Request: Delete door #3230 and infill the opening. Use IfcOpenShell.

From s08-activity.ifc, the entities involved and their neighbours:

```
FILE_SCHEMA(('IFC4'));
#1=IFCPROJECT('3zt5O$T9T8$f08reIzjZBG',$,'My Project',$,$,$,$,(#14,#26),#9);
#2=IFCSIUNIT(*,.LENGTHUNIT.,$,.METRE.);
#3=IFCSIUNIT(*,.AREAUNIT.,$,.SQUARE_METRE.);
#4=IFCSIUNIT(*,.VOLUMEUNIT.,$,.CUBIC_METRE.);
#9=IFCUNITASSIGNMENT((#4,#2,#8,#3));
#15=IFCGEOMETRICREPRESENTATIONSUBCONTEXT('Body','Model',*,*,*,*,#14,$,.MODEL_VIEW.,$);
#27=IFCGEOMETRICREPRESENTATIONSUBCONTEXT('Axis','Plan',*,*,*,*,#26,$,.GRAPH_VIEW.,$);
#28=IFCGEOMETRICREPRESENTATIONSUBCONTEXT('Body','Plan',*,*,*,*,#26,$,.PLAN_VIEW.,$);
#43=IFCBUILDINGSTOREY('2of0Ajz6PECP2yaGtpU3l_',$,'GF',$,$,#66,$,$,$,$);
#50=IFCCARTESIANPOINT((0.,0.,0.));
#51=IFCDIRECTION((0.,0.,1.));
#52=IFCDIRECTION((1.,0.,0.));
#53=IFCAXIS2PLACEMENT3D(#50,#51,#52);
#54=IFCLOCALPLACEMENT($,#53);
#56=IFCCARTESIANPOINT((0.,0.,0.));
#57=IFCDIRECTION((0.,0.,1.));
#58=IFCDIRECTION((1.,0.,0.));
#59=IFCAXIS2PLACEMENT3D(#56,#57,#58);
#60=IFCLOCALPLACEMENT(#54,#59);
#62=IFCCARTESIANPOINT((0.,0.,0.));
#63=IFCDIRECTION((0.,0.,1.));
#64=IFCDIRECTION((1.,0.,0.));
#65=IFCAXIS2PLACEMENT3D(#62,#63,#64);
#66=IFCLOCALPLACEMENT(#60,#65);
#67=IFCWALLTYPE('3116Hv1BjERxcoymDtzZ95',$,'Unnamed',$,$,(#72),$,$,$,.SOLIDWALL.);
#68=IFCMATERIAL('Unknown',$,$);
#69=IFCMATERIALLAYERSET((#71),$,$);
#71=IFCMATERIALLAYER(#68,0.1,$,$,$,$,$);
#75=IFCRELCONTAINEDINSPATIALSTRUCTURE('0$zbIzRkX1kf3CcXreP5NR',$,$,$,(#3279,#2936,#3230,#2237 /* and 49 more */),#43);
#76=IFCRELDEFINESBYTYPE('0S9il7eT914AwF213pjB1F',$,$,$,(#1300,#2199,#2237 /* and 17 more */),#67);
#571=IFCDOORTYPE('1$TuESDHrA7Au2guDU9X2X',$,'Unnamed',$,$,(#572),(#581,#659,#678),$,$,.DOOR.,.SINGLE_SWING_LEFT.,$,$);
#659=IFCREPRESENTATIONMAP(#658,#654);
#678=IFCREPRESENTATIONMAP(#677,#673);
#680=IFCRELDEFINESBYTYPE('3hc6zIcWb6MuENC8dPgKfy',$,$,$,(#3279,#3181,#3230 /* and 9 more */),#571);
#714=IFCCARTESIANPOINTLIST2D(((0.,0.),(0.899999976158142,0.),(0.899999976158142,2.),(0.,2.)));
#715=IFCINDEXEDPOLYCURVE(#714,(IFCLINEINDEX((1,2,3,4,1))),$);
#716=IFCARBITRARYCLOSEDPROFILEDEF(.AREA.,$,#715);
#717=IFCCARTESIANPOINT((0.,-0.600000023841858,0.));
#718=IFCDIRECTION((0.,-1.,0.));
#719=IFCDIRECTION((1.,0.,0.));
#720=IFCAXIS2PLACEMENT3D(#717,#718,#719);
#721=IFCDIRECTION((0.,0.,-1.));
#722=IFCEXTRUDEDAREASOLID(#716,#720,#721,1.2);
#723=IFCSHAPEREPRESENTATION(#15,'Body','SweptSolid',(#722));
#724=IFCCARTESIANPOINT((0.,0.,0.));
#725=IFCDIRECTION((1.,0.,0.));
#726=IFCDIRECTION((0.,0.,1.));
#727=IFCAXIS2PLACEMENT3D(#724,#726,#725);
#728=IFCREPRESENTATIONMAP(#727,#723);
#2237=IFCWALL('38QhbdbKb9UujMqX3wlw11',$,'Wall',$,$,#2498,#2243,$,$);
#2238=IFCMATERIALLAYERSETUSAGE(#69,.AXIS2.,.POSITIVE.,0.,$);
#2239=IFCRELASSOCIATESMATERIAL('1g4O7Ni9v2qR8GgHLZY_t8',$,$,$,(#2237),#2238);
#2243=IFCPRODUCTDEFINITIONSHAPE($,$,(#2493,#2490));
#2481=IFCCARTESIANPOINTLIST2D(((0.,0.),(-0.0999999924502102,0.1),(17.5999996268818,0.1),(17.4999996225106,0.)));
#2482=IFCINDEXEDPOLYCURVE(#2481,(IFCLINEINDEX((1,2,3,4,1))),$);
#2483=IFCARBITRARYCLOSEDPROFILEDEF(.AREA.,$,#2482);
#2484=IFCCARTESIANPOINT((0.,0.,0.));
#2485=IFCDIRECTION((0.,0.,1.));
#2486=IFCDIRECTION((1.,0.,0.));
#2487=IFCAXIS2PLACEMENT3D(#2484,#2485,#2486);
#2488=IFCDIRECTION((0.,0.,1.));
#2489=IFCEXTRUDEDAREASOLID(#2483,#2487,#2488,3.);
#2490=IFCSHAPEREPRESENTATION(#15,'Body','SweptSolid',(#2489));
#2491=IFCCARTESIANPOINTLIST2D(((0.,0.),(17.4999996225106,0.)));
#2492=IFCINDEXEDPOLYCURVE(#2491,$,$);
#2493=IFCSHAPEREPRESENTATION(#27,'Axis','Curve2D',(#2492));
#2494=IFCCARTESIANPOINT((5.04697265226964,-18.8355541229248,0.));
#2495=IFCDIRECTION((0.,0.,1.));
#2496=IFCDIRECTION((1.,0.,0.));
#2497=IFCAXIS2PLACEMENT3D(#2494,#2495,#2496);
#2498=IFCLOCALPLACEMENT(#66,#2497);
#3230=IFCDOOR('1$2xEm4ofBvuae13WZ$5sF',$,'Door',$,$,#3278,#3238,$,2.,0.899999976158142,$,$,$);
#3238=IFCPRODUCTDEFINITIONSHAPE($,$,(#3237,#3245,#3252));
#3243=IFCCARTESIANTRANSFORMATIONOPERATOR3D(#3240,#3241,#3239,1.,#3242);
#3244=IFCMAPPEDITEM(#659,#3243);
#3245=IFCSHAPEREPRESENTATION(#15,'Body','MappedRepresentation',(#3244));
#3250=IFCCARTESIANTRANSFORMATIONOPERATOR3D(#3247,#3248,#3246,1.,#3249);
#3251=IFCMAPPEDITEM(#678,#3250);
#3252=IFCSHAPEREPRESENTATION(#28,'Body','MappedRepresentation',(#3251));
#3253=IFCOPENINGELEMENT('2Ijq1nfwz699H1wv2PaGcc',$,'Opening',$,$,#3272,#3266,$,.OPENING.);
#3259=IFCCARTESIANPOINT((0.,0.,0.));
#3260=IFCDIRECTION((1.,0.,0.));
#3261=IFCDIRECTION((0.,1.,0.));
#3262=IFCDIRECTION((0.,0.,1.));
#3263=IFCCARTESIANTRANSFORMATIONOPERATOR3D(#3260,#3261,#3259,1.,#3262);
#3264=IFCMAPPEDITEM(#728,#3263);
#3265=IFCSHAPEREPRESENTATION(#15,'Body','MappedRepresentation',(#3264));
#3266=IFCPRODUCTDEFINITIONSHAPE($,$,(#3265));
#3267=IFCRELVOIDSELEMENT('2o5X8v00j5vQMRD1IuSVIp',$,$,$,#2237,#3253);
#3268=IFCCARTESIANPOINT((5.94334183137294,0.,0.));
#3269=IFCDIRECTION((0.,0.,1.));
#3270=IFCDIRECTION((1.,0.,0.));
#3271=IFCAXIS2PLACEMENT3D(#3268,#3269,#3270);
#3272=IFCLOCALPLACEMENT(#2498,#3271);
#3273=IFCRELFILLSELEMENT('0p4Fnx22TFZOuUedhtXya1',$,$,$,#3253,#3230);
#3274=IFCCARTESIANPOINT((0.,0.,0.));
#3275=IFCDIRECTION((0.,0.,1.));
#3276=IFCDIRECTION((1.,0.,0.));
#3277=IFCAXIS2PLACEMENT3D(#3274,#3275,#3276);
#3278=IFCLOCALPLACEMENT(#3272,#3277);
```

```python
import ifcopenshell
import ifcopenshell.api.feature
import ifcopenshell.api.root
import ifcopenshell.geom
import ifcopenshell.util.shape

model = ifcopenshell.open("s08-activity.ifc")
settings = ifcopenshell.geom.settings()


def volume(element):
    """Net volume in cubic metres, openings subtracted."""
    shape = ifcopenshell.geom.create_shape(settings, element)
    return ifcopenshell.util.shape.get_volume(shape.geometry)


door = model.by_id(3230)
opening = door.FillsVoids[0].RelatingOpeningElement
wall = opening.VoidsElements[0].RelatingBuildingElement
before = volume(wall)

ifcopenshell.api.root.remove_product(model, product=door)
ifcopenshell.api.feature.remove_feature(model, feature=opening)

after = volume(wall)

print(f"wall volume {before:.3f} -> {after:.3f} m3")

model.write("s08-activity_updated.ifc")
```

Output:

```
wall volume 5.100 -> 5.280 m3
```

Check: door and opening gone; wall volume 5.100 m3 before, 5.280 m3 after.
